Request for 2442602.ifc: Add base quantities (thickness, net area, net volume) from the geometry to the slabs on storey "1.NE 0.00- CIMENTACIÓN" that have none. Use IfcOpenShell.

First a look at what the model holds.

```python
import ifcopenshell
import ifcopenshell.util.element
import ifcopenshell.util.unit

model = ifcopenshell.open("2442602.ifc")
print(model.schema)
for unit_type in ("LENGTHUNIT", "AREAUNIT", "VOLUMEUNIT"):
    print(unit_type, ifcopenshell.util.unit.calculate_unit_scale(model, unit_type))
storey = next(s for s in model.by_type("IfcBuildingStorey") if s.Name == "1.NE 0.00- CIMENTACIÓN")
slabs = [e for e in ifcopenshell.util.element.get_decomposition(storey) if e.is_a("IfcSlab")]
for e in sorted(slabs, key=lambda e: e.id()):
    print(e.id(), e.is_a(), e.Name, list(ifcopenshell.util.element.get_psets(e, qtos_only=True)), sep=" | ")
```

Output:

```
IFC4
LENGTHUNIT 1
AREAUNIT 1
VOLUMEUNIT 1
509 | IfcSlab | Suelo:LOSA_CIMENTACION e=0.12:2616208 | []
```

```python
import ifcopenshell
import ifcopenshell.api.pset
import ifcopenshell.geom
import ifcopenshell.util.element
import ifcopenshell.util.shape
import ifcopenshell.util.unit

model = ifcopenshell.open("2442602.ifc")
unit_scale = ifcopenshell.util.unit.calculate_unit_scale(model)
area_scale = ifcopenshell.util.unit.calculate_unit_scale(model, "AREAUNIT")
volume_scale = ifcopenshell.util.unit.calculate_unit_scale(model, "VOLUMEUNIT")
settings = ifcopenshell.geom.settings()

storey = next(s for s in model.by_type("IfcBuildingStorey") if s.Name == "1.NE 0.00- CIMENTACIÓN")
slabs = [e for e in ifcopenshell.util.element.get_decomposition(storey) if e.is_a("IfcSlab")]

for e in sorted(slabs, key=lambda e: e.id()):
    if ifcopenshell.util.element.get_psets(e, qtos_only=True, should_inherit=False):
        continue
    # Geometry comes back in metres, in the element's own axes.
    shape = ifcopenshell.geom.create_shape(settings, e)
    values = {
        "Width": ifcopenshell.util.shape.get_z(shape.geometry) / unit_scale,
        "NetArea": ifcopenshell.util.shape.get_footprint_area(shape.geometry) / area_scale,
        "NetVolume": ifcopenshell.util.shape.get_volume(shape.geometry) / volume_scale,
    }
    qto = ifcopenshell.api.pset.add_qto(model, product=e, name="Qto_SlabBaseQuantities")
    ifcopenshell.api.pset.edit_qto(model, qto=qto, properties=values)
    print(e.id(), {k: round(v, 3) for k, v in values.items()})

model.write("2442602_updated.ifc")
```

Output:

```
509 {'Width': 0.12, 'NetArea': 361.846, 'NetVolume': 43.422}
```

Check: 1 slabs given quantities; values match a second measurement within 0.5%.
